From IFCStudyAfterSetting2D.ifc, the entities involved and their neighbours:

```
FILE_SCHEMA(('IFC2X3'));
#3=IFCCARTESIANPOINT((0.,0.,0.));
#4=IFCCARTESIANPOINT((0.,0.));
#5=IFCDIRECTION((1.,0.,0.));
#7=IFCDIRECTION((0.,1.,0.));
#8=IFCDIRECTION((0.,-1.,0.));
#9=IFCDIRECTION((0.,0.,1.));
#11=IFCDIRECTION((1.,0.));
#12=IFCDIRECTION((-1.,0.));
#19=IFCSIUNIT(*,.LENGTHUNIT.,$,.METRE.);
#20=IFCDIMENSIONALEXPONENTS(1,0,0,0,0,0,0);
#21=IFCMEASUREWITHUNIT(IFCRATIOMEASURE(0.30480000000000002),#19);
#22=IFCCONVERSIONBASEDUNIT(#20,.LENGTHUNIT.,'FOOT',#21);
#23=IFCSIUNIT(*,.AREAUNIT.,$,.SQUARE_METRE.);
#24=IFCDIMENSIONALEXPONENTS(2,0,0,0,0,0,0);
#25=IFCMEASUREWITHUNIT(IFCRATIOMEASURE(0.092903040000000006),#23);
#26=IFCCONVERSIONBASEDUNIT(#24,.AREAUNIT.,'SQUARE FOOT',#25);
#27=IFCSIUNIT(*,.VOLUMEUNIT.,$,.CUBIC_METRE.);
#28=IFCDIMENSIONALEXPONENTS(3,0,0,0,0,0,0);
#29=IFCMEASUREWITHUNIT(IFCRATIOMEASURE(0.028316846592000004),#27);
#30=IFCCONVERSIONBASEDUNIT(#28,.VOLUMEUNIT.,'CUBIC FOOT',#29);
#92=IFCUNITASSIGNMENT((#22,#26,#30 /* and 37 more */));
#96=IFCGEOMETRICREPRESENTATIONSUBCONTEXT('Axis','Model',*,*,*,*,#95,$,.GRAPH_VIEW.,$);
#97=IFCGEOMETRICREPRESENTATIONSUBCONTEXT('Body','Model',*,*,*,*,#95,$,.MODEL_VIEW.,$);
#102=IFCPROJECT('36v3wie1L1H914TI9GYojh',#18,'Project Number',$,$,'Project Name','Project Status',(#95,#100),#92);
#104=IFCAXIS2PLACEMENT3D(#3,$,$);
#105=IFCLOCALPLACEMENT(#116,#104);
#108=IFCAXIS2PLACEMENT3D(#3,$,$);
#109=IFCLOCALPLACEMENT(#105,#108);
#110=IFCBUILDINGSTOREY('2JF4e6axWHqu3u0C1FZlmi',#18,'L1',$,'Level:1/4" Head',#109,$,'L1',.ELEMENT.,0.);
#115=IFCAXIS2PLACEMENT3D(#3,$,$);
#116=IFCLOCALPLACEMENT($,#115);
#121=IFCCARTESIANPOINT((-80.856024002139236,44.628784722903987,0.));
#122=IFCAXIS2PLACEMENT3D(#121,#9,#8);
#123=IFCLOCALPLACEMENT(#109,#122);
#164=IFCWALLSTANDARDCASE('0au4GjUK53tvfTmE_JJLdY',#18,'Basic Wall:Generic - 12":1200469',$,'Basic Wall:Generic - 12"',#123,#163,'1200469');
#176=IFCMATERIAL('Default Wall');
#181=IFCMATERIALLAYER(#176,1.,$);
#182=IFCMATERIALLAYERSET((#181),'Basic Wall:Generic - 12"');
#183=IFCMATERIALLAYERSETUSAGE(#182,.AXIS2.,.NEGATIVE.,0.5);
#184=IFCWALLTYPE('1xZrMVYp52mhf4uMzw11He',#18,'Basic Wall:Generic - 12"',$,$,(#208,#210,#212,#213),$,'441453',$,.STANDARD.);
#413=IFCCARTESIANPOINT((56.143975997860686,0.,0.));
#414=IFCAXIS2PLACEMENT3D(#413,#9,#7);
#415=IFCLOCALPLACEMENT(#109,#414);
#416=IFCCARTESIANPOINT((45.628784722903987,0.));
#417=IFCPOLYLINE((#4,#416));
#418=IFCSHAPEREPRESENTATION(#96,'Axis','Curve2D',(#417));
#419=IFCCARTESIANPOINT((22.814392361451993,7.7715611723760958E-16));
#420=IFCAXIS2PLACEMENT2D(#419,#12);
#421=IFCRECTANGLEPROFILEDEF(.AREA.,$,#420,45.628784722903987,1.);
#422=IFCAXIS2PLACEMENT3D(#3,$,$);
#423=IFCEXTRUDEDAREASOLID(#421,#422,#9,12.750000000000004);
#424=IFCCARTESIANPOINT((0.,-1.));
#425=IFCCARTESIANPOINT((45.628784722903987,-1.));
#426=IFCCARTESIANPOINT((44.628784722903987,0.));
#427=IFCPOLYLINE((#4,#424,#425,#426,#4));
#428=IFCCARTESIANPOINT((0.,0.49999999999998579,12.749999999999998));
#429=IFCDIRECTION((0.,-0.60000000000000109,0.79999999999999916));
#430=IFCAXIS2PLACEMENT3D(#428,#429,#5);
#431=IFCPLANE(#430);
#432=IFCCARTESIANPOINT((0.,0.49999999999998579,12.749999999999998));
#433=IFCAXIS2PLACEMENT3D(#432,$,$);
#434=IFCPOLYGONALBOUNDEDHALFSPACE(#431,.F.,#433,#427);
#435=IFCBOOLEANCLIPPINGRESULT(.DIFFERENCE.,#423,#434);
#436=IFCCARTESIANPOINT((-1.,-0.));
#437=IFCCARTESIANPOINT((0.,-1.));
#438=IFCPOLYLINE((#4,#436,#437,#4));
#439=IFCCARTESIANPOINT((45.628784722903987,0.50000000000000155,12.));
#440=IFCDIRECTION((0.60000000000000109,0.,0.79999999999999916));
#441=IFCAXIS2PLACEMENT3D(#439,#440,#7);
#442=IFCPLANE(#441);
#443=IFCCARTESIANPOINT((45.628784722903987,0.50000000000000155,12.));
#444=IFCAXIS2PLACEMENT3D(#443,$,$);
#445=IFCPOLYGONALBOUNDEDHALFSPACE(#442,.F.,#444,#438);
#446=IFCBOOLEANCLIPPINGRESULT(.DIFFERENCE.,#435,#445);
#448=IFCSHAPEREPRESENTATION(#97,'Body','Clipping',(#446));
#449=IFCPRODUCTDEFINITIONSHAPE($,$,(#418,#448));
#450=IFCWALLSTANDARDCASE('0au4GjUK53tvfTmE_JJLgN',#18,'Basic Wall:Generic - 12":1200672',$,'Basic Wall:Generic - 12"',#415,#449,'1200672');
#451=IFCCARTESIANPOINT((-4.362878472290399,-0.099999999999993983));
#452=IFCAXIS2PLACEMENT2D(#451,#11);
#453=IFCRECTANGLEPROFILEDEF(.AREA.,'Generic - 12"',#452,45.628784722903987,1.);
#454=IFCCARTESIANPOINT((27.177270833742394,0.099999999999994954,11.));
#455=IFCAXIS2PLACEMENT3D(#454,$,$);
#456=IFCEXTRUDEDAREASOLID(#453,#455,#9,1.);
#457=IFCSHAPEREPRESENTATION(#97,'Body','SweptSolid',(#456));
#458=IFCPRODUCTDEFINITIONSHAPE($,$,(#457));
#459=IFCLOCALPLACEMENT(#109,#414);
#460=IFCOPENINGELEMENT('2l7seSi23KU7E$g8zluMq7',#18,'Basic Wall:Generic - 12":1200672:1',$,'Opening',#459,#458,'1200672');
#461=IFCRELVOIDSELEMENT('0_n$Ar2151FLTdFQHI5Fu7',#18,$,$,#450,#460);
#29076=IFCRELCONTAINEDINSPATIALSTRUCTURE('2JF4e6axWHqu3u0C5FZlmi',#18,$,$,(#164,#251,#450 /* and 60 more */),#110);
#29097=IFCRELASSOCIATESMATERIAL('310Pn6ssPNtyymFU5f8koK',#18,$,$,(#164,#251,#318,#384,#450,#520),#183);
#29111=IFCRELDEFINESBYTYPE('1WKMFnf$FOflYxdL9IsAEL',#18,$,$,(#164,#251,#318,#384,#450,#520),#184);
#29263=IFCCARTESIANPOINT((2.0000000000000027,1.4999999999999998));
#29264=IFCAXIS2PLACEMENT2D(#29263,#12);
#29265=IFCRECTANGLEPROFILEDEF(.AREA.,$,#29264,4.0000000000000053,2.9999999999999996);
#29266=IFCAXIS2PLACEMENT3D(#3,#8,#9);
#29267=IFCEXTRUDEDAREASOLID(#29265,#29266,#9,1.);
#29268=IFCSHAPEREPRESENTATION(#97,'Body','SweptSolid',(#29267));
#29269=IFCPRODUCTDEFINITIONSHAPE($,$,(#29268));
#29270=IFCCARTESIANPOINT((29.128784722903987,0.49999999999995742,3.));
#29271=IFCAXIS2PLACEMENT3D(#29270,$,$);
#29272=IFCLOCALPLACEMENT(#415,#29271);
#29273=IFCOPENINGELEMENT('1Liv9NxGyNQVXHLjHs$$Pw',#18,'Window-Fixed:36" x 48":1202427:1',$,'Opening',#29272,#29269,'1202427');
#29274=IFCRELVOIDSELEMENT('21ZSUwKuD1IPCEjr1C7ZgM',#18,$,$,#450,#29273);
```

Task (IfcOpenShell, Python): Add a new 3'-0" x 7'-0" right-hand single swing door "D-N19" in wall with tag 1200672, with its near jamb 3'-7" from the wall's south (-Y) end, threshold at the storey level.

```python
import numpy as np
import ifcopenshell
import ifcopenshell.api.feature
import ifcopenshell.api.geometry
import ifcopenshell.api.root
import ifcopenshell.api.spatial
import ifcopenshell.api.type
import ifcopenshell.geom
import ifcopenshell.util.element
import ifcopenshell.util.placement
import ifcopenshell.util.representation
import ifcopenshell.util.shape
import ifcopenshell.util.unit

model = ifcopenshell.open("IFCStudyAfterSetting2D.ifc")
unit_scale = ifcopenshell.util.unit.calculate_unit_scale(model)
settings = ifcopenshell.geom.settings()


def volume(element):
    """Net volume in cubic metres, openings subtracted."""
    shape = ifcopenshell.geom.create_shape(settings, element)
    return ifcopenshell.util.shape.get_volume(shape.geometry)


wall = model.by_guid("0au4GjUK53tvfTmE_JJLgN")
storey = ifcopenshell.util.element.get_container(wall, ifc_class="IfcBuildingStorey")
context = ifcopenshell.util.representation.get_context(model, "Model", "Body", "MODEL_VIEW")
before = volume(wall)

width, height, from_end, sill = 0.9144, 2.1336, 1.0922, 0.0  # metres

# The wall runs along its own X axis, and the end named is its -X end.
wall_shape = ifcopenshell.geom.create_shape(settings, wall)
x, y, z = ifcopenshell.util.shape.get_vertices(wall_shape.geometry).T
start = x.min() + from_end
face, thickness = float(y.min()), float(y.max() - y.min())
wall_matrix = ifcopenshell.util.placement.get_local_placement(wall.ObjectPlacement)
level = ifcopenshell.util.placement.get_local_placement(storey.ObjectPlacement)[2, 3]


def in_wall(x, y):
    """Placement at x, y metres in the wall's axes, at sill height."""
    matrix = wall_matrix.copy()
    matrix[:, 3] = wall_matrix @ np.array([x / unit_scale, y / unit_scale, 0.0, 1.0])
    matrix[2, 3] = level + sill / unit_scale
    return matrix


# Opening: a box that overshoots both wall faces by 50 mm.
opening = ifcopenshell.api.root.create_entity(model, ifc_class="IfcOpeningElement")
box = ifcopenshell.api.geometry.add_wall_representation(
    model, context=context, length=width, height=height, thickness=thickness + 0.1
)
ifcopenshell.api.geometry.assign_representation(model, product=opening, representation=box)
ifcopenshell.api.geometry.edit_object_placement(model, product=opening, matrix=in_wall(start, face - 0.05), is_si=False)
ifcopenshell.api.feature.add_feature(model, feature=opening, element=wall)

door = ifcopenshell.api.root.create_entity(model, ifc_class="IfcDoor", name="D-N19")
door.OverallWidth, door.OverallHeight = width / unit_scale, height / unit_scale
body = ifcopenshell.api.geometry.add_door_representation(
    model,
    context=context,
    overall_width=door.OverallWidth,
    overall_height=door.OverallHeight,
    operation_type="SINGLE_SWING_RIGHT",
    lining_properties={"LiningDepth": thickness / unit_scale, "ThresholdDepth": thickness / unit_scale},
)
ifcopenshell.api.geometry.assign_representation(model, product=door, representation=body)
ifcopenshell.api.spatial.assign_container(model, products=[door], relating_structure=storey)
fills = ifcopenshell.api.feature.add_filling(model, opening=opening, element=door)
fills.OwnerHistory = door.OwnerHistory  # required in IFC2X3

# IFC2X3 keeps the operation on the door style.
style = ifcopenshell.api.root.create_entity(model, ifc_class="IfcDoorStyle", name="D-N19")
style.OperationType, style.ConstructionType = "SINGLE_SWING_RIGHT", "NOTDEFINED"
style.ParameterTakesPrecedence = style.Sizeable = False
ifcopenshell.api.type.assign_type(model, related_objects=[door], relating_type=style)

# The lining spans the wall, so the door starts at the wall face.
ifcopenshell.api.geometry.edit_object_placement(model, product=door, matrix=in_wall(start, face), is_si=False)

after = volume(wall)

print(f"wall volume {before:.3f} -> {after:.3f} m3")

model.write("IFCStudyAfterSetting2D_v2.ifc")
```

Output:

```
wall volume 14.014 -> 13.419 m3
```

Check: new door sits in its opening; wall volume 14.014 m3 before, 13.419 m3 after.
